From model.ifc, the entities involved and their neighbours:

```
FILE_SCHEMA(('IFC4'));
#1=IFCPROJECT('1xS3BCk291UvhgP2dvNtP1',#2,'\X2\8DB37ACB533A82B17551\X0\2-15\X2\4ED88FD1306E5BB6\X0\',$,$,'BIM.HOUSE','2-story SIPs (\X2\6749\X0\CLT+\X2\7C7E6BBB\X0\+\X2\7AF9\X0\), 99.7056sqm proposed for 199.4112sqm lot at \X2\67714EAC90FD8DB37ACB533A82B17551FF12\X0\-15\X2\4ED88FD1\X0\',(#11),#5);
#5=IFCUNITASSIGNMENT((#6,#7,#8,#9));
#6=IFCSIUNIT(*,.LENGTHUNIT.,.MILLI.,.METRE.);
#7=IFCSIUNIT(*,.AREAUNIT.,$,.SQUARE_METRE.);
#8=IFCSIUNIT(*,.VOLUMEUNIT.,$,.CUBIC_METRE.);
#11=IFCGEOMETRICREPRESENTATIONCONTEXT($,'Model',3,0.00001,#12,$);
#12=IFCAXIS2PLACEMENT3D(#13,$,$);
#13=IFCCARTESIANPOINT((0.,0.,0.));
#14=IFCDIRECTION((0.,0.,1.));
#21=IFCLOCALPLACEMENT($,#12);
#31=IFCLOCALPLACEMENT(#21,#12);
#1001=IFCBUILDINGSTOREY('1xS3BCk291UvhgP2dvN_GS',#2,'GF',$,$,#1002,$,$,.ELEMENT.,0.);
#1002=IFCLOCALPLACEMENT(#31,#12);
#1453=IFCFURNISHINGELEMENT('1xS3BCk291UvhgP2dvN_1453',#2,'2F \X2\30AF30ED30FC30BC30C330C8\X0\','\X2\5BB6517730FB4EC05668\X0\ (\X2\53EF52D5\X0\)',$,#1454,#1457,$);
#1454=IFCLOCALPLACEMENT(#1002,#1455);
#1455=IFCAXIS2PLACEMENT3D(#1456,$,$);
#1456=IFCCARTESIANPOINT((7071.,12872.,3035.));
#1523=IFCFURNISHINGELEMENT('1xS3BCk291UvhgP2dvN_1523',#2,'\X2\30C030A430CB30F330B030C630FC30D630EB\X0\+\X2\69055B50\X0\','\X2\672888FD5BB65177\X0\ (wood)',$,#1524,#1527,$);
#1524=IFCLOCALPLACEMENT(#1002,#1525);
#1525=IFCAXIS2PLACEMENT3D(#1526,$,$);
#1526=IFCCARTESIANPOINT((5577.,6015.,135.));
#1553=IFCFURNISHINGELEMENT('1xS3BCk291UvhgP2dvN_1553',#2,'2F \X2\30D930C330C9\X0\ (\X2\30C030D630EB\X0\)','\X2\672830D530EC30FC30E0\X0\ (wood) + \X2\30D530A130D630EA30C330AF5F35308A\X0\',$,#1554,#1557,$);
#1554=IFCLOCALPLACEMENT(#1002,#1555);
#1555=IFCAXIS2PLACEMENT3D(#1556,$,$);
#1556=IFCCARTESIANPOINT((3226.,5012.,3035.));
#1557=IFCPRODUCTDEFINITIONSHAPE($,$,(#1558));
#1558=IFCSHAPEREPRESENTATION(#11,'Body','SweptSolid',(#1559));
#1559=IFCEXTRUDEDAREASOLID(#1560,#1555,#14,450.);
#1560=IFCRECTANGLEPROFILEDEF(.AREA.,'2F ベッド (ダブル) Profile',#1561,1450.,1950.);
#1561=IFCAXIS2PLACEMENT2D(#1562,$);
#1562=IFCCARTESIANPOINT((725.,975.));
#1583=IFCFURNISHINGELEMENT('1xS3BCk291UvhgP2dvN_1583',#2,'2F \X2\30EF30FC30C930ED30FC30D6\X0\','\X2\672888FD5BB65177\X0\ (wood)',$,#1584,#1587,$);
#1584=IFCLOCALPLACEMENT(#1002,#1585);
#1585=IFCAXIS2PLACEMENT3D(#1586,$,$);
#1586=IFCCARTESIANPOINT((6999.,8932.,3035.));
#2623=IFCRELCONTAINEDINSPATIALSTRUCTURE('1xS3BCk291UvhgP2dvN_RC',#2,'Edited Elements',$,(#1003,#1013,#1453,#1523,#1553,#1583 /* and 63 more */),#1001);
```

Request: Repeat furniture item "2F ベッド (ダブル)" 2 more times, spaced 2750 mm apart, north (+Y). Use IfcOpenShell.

```python
import numpy as np
import ifcopenshell
import ifcopenshell.api.geometry
import ifcopenshell.api.root
import ifcopenshell.util.element
import ifcopenshell.util.placement
import ifcopenshell.util.unit

model = ifcopenshell.open("model.ifc")
unit_scale = ifcopenshell.util.unit.calculate_unit_scale(model)


def reuse_history(source, copy):
    """copy_class also copies each property set's owner history, people and application; keep the originals."""
    for rel in copy.IsDefinedBy:
        if rel.is_a("IfcRelDefinesByProperties") and (history := rel.RelatingPropertyDefinition.OwnerHistory):
            rel.RelatingPropertyDefinition.OwnerHistory = source.OwnerHistory
            ifcopenshell.util.element.remove_deep2(model, history)


source = model.by_id(1553)
base = ifcopenshell.util.placement.get_local_placement(source.ObjectPlacement)
step = np.array([0.0, 1.0, 0.0]) * 2.75 / unit_scale

for i in range(1, 3):
    copy = ifcopenshell.api.root.copy_class(model, product=source)
    copy.Representation = ifcopenshell.util.element.copy_deep(
        model, source.Representation, exclude=["IfcGeometricRepresentationContext", "IfcRepresentationMap"]
    )
    reuse_history(source, copy)
    matrix = base.copy()
    matrix[:3, 3] += i * step
    print("added at", matrix[:3, 3].round(3) + 0.0)
    ifcopenshell.api.geometry.edit_object_placement(model, product=copy, matrix=matrix, is_si=False)

model.write("model-out.ifc")
```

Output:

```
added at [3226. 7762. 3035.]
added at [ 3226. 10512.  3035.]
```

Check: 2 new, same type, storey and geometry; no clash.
